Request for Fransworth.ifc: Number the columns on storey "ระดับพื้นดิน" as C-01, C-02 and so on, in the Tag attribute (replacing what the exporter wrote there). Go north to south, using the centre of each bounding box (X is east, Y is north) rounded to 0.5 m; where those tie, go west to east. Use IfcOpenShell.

First a look at what the model holds.

```python
import ifcopenshell
import ifcopenshell.util.element
import ifcopenshell.util.placement

model = ifcopenshell.open("Fransworth.ifc")
print(model.schema)
storey = next(s for s in model.by_type("IfcBuildingStorey") if s.Name == "ระดับพื้นดิน")
columns = [e for e in ifcopenshell.util.element.get_decomposition(storey) if e.is_a("IfcColumn")]
for e in sorted(columns, key=lambda e: e.id()):
    origin = ifcopenshell.util.placement.get_local_placement(e.ObjectPlacement)[:3, 3]
    print(e.id(), e.Tag, e.Name, origin.round(2) + 0.0, sep=" | ")
```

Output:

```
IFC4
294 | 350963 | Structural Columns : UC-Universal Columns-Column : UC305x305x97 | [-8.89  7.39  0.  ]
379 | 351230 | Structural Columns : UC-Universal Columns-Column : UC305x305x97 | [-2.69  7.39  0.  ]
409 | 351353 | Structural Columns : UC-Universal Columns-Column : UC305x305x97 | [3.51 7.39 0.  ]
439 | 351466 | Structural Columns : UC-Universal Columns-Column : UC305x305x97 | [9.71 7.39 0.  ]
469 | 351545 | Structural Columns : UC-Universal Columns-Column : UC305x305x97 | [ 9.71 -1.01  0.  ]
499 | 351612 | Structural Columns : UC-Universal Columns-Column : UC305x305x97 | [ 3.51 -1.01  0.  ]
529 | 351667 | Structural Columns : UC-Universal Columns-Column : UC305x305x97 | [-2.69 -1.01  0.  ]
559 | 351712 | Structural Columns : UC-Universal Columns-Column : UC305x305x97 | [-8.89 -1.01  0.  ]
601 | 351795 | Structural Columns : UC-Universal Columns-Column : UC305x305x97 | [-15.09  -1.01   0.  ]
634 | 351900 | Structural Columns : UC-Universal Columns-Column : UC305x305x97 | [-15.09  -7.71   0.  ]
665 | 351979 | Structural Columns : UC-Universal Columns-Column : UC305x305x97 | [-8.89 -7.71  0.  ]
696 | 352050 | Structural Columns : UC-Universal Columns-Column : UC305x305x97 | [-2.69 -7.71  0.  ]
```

```python
import ifcopenshell
import ifcopenshell.geom
import ifcopenshell.util.element
import ifcopenshell.util.shape

model = ifcopenshell.open("Fransworth.ifc")
settings = ifcopenshell.geom.settings()
settings.set("use-world-coords", True)


def centre(element):
    shape = ifcopenshell.geom.create_shape(settings, element)
    return ifcopenshell.util.shape.get_bbox_centroid(shape.geometry)


storey = next(s for s in model.by_type("IfcBuildingStorey") if s.Name == "ระดับพื้นดิน")
columns = [e for e in ifcopenshell.util.element.get_decomposition(storey) if e.is_a("IfcColumn")]

# Insertion points can sit at a corner or the storey origin, so sort by the geometry (in metres).
centres = {e: centre(e) for e in columns}
columns.sort(key=lambda e: (-round(centres[e][1] / 0.5), centres[e][0]))

for i, e in enumerate(columns, start=1):
    number = f"C-{i:02d}"
    e.Tag = number
    print(e.id(), number)

model.write("Fransworth_updated.ifc")
```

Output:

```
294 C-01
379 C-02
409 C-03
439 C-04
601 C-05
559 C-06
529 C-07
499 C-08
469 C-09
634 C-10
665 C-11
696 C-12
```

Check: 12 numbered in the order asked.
